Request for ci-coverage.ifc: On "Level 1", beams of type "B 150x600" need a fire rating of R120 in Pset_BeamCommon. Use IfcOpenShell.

First a look at what the model holds.

```python
import ifcopenshell
import ifcopenshell.util.element

model = ifcopenshell.open("ci-coverage.ifc")
print(model.schema)
storey = next(s for s in model.by_type("IfcBuildingStorey") if s.Name == "Level 1")
beams = [e for e in ifcopenshell.util.element.get_decomposition(storey) if e.is_a("IfcBeam")]
seen = {}
for e in beams:
    element_type = ifcopenshell.util.element.get_type(e)
    key = (element_type.Name if element_type != e and element_type else None, ifcopenshell.util.element.get_pset(e, "Pset_BeamCommon", "FireRating"))
    seen[key] = seen.get(key, 0) + 1
for (name, value), count in sorted(seen.items(), key=str):
    print(count, "x", name, "|", value)
```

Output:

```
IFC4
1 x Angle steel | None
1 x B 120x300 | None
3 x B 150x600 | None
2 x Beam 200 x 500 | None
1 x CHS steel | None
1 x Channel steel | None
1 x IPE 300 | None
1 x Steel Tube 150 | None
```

```python
import ifcopenshell
import ifcopenshell.api.pset
import ifcopenshell.util.element

model = ifcopenshell.open("ci-coverage.ifc")

storey = next(s for s in model.by_type("IfcBuildingStorey") if s.Name == "Level 1")
beams = [e for e in ifcopenshell.util.element.get_decomposition(storey) if e.is_a("IfcBeam")]

count = 0
for e in beams:
    element_type = ifcopenshell.util.element.get_type(e)
    if element_type in (None, e) or element_type.Name != "B 150x600":
        continue
    # add_pset returns the element's existing set when there is one.
    pset = ifcopenshell.api.pset.add_pset(model, product=e, name="Pset_BeamCommon")
    ifcopenshell.api.pset.edit_pset(model, pset=pset, properties={"FireRating": "R120"})
    count += 1

print(count, "beams updated")

model.write("ci-coverage_updated.ifc")
```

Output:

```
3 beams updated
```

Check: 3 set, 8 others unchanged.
